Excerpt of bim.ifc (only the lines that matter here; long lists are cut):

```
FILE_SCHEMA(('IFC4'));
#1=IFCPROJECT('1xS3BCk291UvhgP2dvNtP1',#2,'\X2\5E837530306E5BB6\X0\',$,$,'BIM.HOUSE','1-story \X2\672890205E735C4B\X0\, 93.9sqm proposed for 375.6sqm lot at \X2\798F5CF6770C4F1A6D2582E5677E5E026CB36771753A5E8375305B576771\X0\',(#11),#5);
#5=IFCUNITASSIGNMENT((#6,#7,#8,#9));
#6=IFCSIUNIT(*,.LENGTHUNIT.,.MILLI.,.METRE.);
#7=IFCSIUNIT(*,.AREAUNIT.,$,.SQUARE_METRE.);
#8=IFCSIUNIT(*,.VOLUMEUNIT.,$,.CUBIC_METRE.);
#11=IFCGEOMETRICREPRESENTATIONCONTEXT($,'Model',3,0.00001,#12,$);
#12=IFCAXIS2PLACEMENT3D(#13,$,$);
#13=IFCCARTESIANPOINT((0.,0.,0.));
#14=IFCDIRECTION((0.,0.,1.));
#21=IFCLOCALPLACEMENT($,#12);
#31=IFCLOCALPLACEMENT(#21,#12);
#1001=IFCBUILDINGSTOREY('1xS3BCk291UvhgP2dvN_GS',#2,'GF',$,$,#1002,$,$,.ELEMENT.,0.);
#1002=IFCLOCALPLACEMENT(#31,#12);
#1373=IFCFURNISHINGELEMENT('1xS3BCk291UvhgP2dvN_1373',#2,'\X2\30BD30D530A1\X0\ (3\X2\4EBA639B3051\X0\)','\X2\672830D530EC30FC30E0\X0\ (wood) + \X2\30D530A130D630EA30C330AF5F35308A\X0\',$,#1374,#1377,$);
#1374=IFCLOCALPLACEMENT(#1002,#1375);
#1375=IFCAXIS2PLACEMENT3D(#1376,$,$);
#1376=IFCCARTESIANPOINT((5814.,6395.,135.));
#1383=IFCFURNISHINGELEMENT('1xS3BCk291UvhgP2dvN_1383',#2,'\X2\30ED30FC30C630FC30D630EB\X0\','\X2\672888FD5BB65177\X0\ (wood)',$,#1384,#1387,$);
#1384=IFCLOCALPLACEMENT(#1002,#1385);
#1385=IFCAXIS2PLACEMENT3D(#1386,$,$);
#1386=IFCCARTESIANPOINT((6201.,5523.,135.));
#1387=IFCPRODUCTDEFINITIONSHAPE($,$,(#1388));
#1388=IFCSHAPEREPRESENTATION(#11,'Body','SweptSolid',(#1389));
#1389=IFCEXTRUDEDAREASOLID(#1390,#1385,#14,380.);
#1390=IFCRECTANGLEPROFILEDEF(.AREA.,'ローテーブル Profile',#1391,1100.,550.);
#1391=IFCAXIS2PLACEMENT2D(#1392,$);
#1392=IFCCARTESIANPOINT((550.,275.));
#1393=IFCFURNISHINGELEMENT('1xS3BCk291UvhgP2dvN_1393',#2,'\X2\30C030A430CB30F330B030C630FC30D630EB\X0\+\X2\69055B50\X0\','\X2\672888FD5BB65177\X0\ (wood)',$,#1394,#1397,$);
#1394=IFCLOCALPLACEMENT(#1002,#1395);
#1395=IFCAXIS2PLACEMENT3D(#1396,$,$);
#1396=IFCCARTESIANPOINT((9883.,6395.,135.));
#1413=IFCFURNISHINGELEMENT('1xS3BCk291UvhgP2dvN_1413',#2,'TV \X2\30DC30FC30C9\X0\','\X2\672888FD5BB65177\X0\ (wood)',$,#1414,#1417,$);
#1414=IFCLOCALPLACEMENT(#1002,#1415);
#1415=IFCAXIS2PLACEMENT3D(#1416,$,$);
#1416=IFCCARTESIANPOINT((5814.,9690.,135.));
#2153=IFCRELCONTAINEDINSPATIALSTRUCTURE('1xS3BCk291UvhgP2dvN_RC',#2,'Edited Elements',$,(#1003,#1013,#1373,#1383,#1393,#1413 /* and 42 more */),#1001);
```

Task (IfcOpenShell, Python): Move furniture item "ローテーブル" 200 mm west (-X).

```python
import ifcopenshell
import ifcopenshell.api.geometry
import ifcopenshell.util.placement

model = ifcopenshell.open("bim.ifc")

item = model.by_guid("1xS3BCk291UvhgP2dvN_1383")
matrix = ifcopenshell.util.placement.get_local_placement(item.ObjectPlacement)
matrix[0, 3] -= 200.0
ifcopenshell.api.geometry.edit_object_placement(model, product=item, matrix=matrix, is_si=False)

print(ifcopenshell.util.placement.get_local_placement(item.ObjectPlacement).round(3) + 0.0)

model.write("bim_rev.ifc")
```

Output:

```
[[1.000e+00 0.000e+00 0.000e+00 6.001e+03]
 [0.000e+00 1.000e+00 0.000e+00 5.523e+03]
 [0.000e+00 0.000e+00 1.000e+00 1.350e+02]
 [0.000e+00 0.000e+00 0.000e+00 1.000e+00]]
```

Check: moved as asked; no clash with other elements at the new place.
